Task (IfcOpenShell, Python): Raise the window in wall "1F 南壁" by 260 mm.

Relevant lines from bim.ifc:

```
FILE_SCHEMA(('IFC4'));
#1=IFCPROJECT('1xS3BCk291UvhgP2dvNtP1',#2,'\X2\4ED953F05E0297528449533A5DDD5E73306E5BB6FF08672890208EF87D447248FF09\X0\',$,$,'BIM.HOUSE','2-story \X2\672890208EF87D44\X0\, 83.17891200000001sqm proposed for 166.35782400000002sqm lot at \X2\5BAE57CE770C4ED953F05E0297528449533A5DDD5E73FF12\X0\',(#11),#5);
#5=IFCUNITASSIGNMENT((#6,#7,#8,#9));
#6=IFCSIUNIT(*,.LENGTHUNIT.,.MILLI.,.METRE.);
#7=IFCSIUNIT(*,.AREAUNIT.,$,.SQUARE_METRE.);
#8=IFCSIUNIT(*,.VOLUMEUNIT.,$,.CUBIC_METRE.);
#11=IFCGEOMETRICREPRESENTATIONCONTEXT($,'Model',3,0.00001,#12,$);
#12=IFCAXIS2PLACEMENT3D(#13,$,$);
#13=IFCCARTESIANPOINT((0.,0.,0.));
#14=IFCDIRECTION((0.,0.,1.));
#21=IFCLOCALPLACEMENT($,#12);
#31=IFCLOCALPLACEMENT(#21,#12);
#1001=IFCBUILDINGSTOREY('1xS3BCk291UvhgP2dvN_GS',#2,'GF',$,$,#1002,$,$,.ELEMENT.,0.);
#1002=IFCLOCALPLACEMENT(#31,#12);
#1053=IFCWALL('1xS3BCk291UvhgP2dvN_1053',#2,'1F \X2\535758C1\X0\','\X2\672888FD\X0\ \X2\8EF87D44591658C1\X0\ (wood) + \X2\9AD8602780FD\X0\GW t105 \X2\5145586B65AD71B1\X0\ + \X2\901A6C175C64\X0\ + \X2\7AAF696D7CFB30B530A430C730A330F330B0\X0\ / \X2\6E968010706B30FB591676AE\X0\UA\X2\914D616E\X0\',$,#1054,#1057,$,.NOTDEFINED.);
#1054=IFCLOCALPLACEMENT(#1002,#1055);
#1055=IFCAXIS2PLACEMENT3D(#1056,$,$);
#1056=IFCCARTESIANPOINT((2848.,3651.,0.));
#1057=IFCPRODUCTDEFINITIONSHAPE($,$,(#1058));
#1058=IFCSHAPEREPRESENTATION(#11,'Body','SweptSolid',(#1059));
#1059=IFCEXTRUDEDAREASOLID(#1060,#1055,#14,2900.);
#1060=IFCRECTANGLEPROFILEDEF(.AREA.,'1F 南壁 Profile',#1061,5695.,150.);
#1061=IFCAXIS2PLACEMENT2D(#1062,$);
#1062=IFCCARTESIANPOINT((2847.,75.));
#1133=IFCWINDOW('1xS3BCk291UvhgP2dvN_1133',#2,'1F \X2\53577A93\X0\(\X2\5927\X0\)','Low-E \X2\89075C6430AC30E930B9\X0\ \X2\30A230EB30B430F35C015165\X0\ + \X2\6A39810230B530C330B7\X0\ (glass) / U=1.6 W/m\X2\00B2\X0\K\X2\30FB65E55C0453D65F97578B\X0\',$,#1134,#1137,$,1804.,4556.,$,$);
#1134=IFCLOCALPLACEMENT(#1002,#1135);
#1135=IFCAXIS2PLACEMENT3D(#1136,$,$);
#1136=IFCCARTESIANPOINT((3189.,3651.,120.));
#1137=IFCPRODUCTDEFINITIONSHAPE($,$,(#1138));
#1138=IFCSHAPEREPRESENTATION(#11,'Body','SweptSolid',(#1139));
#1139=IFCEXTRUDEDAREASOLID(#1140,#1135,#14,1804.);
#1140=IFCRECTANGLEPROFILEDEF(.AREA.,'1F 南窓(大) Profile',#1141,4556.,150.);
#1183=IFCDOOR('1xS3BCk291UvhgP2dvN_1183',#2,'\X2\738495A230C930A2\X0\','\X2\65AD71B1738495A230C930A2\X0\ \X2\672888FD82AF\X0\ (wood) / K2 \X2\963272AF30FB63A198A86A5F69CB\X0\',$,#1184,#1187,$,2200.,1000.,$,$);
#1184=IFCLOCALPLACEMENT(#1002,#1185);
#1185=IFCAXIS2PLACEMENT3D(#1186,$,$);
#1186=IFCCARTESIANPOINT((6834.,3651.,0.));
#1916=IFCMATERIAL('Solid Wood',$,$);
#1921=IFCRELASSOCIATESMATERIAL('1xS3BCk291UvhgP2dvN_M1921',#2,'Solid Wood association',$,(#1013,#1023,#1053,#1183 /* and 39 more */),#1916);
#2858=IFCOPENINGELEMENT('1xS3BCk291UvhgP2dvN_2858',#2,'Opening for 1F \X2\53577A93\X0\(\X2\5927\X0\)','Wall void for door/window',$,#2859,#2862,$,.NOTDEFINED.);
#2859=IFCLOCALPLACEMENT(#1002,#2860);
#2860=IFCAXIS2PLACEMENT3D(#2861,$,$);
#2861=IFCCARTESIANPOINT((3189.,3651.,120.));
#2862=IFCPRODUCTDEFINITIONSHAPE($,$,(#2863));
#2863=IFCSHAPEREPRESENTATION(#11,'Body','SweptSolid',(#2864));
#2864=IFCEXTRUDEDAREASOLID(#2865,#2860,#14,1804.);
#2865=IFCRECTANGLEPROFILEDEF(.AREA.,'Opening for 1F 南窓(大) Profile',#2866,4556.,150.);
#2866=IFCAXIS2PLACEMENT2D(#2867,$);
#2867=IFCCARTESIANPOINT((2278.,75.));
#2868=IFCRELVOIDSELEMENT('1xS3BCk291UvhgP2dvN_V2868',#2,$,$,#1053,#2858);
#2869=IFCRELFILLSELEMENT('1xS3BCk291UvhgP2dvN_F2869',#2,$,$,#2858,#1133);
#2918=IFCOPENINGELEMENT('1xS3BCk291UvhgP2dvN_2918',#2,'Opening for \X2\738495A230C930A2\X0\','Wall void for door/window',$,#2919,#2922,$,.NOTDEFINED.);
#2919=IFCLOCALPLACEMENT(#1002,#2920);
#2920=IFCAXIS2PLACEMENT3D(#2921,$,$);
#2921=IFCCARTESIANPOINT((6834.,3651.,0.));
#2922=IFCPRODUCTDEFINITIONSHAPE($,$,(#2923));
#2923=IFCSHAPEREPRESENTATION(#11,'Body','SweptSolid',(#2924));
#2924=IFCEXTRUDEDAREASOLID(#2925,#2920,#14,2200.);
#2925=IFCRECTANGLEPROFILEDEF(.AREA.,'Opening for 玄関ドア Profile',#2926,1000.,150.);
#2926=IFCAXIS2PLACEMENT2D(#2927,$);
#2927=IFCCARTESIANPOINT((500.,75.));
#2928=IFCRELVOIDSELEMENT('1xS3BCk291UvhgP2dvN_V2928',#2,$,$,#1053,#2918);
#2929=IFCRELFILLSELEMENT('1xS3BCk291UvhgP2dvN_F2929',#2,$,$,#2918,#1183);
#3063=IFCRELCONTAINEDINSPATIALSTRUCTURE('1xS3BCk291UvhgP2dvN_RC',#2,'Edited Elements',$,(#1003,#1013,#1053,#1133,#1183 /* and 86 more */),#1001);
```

```python
import numpy as np
import ifcopenshell
import ifcopenshell.api.geometry
import ifcopenshell.util.placement
import ifcopenshell.util.unit

model = ifcopenshell.open("bim.ifc")
unit_scale = ifcopenshell.util.unit.calculate_unit_scale(model)

window = model.by_guid("1xS3BCk291UvhgP2dvN_1133")
opening = window.FillsVoids[0].RelatingOpeningElement
dz = 260.0

shift = np.array([0.0, 0.0, dz])
# The window is not placed relative to its opening, so move both.
for product in (opening, window):
    matrix = ifcopenshell.util.placement.get_local_placement(product.ObjectPlacement)
    matrix[:3, 3] += shift
    ifcopenshell.api.geometry.edit_object_placement(model, product=product, matrix=matrix, is_si=False)

print(f"moved by {dz * unit_scale:+.3f} m")

model.write("bim_rev.ifc")
```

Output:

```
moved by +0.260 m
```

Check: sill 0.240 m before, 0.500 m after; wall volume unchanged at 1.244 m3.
